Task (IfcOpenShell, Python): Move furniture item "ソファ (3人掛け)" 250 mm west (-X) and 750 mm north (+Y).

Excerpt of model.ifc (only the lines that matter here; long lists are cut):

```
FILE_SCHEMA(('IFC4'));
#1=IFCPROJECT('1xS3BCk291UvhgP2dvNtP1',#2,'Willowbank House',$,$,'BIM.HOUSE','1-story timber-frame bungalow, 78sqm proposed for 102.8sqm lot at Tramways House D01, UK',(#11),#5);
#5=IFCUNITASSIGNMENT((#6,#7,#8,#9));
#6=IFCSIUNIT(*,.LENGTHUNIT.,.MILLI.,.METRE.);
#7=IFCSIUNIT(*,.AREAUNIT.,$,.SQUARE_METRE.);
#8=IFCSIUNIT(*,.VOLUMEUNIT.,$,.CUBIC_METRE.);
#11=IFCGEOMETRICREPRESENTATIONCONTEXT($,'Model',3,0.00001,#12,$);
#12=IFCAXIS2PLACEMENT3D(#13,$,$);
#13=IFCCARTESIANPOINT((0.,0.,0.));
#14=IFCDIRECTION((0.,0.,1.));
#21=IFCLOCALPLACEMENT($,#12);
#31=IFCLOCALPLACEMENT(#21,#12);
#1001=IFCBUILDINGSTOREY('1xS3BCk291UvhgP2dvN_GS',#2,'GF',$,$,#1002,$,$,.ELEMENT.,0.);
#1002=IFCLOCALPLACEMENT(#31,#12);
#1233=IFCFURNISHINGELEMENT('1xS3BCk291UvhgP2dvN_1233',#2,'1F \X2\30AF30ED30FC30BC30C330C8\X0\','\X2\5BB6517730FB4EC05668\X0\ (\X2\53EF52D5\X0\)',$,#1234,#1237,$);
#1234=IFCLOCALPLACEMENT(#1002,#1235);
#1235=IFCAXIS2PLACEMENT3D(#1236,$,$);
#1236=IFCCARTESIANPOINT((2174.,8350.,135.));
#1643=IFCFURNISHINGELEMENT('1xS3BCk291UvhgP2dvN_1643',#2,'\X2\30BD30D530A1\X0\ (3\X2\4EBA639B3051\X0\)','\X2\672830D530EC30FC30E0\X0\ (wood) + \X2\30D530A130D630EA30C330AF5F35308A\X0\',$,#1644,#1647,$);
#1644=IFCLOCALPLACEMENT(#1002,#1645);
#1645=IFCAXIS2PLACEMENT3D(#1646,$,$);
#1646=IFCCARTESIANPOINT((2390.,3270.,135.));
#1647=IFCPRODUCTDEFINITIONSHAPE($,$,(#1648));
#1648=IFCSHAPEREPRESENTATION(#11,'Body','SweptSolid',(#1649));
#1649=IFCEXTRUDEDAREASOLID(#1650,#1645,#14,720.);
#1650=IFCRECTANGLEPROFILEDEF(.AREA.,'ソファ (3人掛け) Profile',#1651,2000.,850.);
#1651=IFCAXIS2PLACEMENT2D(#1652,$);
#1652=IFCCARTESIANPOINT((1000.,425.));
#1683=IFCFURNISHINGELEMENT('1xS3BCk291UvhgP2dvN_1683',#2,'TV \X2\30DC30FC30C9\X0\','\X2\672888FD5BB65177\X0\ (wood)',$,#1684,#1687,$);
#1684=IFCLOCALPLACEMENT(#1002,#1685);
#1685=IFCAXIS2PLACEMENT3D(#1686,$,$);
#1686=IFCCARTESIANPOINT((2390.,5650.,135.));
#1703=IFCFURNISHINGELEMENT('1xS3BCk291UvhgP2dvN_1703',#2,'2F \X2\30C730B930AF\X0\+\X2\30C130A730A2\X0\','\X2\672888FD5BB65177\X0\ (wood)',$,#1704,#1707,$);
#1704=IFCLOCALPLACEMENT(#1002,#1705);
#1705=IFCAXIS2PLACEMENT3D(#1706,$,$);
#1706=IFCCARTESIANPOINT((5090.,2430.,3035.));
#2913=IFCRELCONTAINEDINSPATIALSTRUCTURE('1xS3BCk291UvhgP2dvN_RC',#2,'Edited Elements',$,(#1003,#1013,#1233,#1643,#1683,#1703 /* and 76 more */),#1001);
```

```python
import ifcopenshell
import ifcopenshell.api.geometry
import ifcopenshell.util.placement
import ifcopenshell.util.unit

model = ifcopenshell.open("model.ifc")
unit_scale = ifcopenshell.util.unit.calculate_unit_scale(model)

item = model.by_guid("1xS3BCk291UvhgP2dvN_1643")
matrix = ifcopenshell.util.placement.get_local_placement(item.ObjectPlacement)
matrix[0, 3] -= 0.25 / unit_scale
matrix[1, 3] += 0.75 / unit_scale
ifcopenshell.api.geometry.edit_object_placement(model, product=item, matrix=matrix, is_si=False)

print(ifcopenshell.util.placement.get_local_placement(item.ObjectPlacement).round(3) + 0.0)

model.write("model-out.ifc")
```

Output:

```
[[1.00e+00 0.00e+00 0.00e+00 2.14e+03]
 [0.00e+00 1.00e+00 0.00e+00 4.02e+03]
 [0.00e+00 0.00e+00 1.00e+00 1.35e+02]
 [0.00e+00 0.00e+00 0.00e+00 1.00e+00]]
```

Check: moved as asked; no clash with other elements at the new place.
